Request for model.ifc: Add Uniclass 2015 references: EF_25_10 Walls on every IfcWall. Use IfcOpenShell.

First a look at what the model holds.

```python
import ifcopenshell

model = ifcopenshell.open("model.ifc")
print(model.schema)
print("classifications:", [c.Name for c in model.by_type("IfcClassification")])
for ifc_class in ("IfcDoor", "IfcRoof", "IfcStair", "IfcWall", "IfcWindow"):
    print(ifc_class, len(model.by_type(ifc_class)))
```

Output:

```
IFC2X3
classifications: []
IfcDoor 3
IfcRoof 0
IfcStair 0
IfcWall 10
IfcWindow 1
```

```python
import ifcopenshell
import ifcopenshell.api.classification

model = ifcopenshell.open("model.ifc")

# IFC2X3 requires Source and Edition and has no link from the project to the system.
system = model.create_entity("IfcClassification", Source="NBS", Edition="2015", Name="Uniclass 2015")

codes = {
    "IfcWall": ("EF_25_10", "Walls"),
}
for ifc_class, (code, name) in codes.items():
    products = model.by_type(ifc_class)
    ifcopenshell.api.classification.add_reference(
        model, products=products, classification=system, identification=code, name=name
    )
    print(code, len(products))

model.write("model_updated.ifc")
```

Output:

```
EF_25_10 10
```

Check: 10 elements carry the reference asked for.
